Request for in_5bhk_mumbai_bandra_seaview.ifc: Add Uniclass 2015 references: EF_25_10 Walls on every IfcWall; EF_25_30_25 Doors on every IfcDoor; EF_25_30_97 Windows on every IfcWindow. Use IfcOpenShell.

First a look at what the model holds.

```python
import ifcopenshell

model = ifcopenshell.open("in_5bhk_mumbai_bandra_seaview.ifc")
print(model.schema)
print("classifications:", [c.Name for c in model.by_type("IfcClassification")])
for ifc_class in ("IfcDoor", "IfcRoof", "IfcStair", "IfcWall", "IfcWindow"):
    print(ifc_class, len(model.by_type(ifc_class)))
```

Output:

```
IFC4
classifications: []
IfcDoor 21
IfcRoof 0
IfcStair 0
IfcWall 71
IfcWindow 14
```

```python
import ifcopenshell
import ifcopenshell.api.classification

model = ifcopenshell.open("in_5bhk_mumbai_bandra_seaview.ifc")

system = ifcopenshell.api.classification.add_classification(model, classification="Uniclass 2015")

codes = {
    "IfcWall": ("EF_25_10", "Walls"),
    "IfcDoor": ("EF_25_30_25", "Doors"),
    "IfcWindow": ("EF_25_30_97", "Windows"),
}
for ifc_class, (code, name) in codes.items():
    products = model.by_type(ifc_class)
    ifcopenshell.api.classification.add_reference(
        model, products=products, classification=system, identification=code, name=name
    )
    print(code, len(products))

model.write("in_5bhk_mumbai_bandra_seaview_updated.ifc")
```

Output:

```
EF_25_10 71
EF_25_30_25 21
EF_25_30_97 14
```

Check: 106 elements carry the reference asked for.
